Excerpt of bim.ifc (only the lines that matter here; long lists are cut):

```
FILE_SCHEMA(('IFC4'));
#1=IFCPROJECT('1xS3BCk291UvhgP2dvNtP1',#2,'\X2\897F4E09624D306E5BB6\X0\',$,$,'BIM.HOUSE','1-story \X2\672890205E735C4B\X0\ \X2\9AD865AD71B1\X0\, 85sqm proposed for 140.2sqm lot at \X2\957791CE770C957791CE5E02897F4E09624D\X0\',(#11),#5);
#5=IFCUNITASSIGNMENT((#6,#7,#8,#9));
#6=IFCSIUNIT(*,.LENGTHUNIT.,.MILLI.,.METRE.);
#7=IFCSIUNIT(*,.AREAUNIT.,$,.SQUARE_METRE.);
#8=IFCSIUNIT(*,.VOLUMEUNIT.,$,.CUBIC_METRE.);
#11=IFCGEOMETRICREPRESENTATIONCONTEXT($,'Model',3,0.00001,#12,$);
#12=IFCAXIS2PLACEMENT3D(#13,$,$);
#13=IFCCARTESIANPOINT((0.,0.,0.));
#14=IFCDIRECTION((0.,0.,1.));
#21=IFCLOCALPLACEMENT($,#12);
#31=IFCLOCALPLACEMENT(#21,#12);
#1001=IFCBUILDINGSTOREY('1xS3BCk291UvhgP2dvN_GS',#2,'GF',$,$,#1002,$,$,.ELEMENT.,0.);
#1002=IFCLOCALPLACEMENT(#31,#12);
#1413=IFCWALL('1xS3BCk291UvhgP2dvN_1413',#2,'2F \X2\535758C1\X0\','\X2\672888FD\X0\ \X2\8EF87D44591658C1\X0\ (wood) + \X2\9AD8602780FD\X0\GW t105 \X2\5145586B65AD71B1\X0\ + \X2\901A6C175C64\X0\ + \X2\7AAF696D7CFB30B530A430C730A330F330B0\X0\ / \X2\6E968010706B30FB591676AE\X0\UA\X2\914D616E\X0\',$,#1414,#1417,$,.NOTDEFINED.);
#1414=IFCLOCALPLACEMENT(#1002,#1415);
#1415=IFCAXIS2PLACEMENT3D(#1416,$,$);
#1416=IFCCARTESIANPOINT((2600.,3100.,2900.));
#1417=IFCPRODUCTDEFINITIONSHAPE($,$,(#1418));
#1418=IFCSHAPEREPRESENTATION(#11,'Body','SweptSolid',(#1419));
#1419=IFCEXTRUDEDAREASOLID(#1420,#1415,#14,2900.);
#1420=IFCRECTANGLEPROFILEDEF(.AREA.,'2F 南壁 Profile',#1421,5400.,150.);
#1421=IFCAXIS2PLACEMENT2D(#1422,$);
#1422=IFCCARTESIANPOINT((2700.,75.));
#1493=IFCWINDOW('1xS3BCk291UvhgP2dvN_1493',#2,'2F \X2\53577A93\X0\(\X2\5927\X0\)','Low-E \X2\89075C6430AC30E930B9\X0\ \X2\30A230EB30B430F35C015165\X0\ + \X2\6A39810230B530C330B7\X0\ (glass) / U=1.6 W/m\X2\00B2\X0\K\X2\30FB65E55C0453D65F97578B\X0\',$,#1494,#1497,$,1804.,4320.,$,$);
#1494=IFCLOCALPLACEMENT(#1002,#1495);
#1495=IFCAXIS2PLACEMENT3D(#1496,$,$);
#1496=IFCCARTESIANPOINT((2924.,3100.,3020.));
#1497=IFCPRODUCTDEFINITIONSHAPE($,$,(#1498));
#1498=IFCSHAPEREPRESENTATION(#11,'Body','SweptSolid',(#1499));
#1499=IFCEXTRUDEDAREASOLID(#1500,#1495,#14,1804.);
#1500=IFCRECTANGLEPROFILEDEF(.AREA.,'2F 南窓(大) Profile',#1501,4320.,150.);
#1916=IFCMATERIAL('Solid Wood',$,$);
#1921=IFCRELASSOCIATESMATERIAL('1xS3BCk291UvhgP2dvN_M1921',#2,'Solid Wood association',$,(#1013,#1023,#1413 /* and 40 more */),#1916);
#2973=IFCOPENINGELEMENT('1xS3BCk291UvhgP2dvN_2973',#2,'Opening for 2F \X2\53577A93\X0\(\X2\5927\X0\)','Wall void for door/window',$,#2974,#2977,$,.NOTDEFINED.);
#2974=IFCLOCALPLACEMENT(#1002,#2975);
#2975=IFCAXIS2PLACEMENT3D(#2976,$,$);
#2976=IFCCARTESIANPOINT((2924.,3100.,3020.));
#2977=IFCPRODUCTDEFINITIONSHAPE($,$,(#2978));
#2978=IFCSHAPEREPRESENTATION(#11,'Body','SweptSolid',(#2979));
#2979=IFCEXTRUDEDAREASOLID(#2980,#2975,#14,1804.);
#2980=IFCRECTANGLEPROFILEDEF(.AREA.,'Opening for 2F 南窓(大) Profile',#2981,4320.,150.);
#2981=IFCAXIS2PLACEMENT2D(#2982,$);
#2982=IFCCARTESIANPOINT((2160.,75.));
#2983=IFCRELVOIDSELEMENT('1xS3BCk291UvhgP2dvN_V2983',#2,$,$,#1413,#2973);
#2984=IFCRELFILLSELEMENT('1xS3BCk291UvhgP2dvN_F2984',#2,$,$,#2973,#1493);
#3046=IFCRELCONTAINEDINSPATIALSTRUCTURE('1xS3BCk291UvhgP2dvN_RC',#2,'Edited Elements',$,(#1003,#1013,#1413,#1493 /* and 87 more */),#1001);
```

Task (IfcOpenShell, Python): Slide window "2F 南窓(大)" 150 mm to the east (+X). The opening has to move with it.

```python
import ifcopenshell
import ifcopenshell.api.geometry
import ifcopenshell.util.placement
import ifcopenshell.util.unit

model = ifcopenshell.open("bim.ifc")
unit_scale = ifcopenshell.util.unit.calculate_unit_scale(model)

window = model.by_guid("1xS3BCk291UvhgP2dvN_1493")
opening = window.FillsVoids[0].RelatingOpeningElement
wall = opening.VoidsElements[0].RelatingBuildingElement

wall_matrix = ifcopenshell.util.placement.get_local_placement(wall.ObjectPlacement)
shift = wall_matrix[:3, 0] * 0.15 / unit_scale
before = ifcopenshell.util.placement.get_local_placement(window.ObjectPlacement)[:3, 3].copy()

# The window is not placed relative to its opening, so move both.
for product in (opening, window):
    matrix = ifcopenshell.util.placement.get_local_placement(product.ObjectPlacement)
    matrix[:3, 3] += shift
    ifcopenshell.api.geometry.edit_object_placement(model, product=product, matrix=matrix, is_si=False)

after = ifcopenshell.util.placement.get_local_placement(window.ObjectPlacement)[:3, 3]
print("window moved by", (after - before).round(3) + 0.0)

model.write("bim_v2.ifc")
```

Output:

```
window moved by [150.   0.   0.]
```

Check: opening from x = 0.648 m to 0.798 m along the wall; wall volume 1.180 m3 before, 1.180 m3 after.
